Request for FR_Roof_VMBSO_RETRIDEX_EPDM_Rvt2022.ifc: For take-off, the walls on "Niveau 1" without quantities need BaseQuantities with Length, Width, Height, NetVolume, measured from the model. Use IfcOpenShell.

First a look at what the model holds.

```python
import ifcopenshell
import ifcopenshell.util.element
import ifcopenshell.util.unit

model = ifcopenshell.open("FR_Roof_VMBSO_RETRIDEX_EPDM_Rvt2022.ifc")
print(model.schema)
for unit_type in ("LENGTHUNIT", "AREAUNIT", "VOLUMEUNIT"):
    print(unit_type, ifcopenshell.util.unit.calculate_unit_scale(model, unit_type))
storey = next(s for s in model.by_type("IfcBuildingStorey") if s.Name == "Niveau 1")
walls = [e for e in ifcopenshell.util.element.get_decomposition(storey) if e.is_a("IfcWall")]
for e in sorted(walls, key=lambda e: e.id()):
    print(e.id(), e.is_a(), e.Name, list(ifcopenshell.util.element.get_psets(e, qtos_only=True)), sep=" | ")
```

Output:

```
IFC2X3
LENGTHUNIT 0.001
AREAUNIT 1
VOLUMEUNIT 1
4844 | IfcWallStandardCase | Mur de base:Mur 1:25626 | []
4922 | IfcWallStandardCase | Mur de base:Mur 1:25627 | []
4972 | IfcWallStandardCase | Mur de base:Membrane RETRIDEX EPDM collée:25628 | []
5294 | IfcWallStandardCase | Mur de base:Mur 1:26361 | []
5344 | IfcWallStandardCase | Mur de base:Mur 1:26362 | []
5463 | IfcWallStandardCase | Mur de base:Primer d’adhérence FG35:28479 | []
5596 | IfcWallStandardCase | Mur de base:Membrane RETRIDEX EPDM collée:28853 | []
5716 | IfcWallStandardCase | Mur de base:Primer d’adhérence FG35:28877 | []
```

```python
import ifcopenshell
import ifcopenshell.api.pset
import ifcopenshell.geom
import ifcopenshell.util.element
import ifcopenshell.util.shape
import ifcopenshell.util.unit

model = ifcopenshell.open("FR_Roof_VMBSO_RETRIDEX_EPDM_Rvt2022.ifc")
unit_scale = ifcopenshell.util.unit.calculate_unit_scale(model)
volume_scale = ifcopenshell.util.unit.calculate_unit_scale(model, "VOLUMEUNIT")
settings = ifcopenshell.geom.settings()

storey = next(s for s in model.by_type("IfcBuildingStorey") if s.Name == "Niveau 1")
walls = [e for e in ifcopenshell.util.element.get_decomposition(storey) if e.is_a("IfcWall")]

for e in sorted(walls, key=lambda e: e.id()):
    if ifcopenshell.util.element.get_psets(e, qtos_only=True, should_inherit=False):
        continue
    # Geometry comes back in metres, in the element's own axes.
    shape = ifcopenshell.geom.create_shape(settings, e)
    values = {
        "Length": ifcopenshell.util.shape.get_x(shape.geometry) / unit_scale,
        "Width": ifcopenshell.util.shape.get_y(shape.geometry) / unit_scale,
        "Height": ifcopenshell.util.shape.get_z(shape.geometry) / unit_scale,
        "NetVolume": ifcopenshell.util.shape.get_volume(shape.geometry) / volume_scale,
    }
    qto = ifcopenshell.api.pset.add_qto(model, product=e, name="BaseQuantities")
    ifcopenshell.api.pset.edit_qto(model, qto=qto, properties=values)
    print(e.id(), {k: round(v, 3) for k, v in values.items()})

model.write("FR_Roof_VMBSO_RETRIDEX_EPDM_Rvt2022_rev.ifc")
```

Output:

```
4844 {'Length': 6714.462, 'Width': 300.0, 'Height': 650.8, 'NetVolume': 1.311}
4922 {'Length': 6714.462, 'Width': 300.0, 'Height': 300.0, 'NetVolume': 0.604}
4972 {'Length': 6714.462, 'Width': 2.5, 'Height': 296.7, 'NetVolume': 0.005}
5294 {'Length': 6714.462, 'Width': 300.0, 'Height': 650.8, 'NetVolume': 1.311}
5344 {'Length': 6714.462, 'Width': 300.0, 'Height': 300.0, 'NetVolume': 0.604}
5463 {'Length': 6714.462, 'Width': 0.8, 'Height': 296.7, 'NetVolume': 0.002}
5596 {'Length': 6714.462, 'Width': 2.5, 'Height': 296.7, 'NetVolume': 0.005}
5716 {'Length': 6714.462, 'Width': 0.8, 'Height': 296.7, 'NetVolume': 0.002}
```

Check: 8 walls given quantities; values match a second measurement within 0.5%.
